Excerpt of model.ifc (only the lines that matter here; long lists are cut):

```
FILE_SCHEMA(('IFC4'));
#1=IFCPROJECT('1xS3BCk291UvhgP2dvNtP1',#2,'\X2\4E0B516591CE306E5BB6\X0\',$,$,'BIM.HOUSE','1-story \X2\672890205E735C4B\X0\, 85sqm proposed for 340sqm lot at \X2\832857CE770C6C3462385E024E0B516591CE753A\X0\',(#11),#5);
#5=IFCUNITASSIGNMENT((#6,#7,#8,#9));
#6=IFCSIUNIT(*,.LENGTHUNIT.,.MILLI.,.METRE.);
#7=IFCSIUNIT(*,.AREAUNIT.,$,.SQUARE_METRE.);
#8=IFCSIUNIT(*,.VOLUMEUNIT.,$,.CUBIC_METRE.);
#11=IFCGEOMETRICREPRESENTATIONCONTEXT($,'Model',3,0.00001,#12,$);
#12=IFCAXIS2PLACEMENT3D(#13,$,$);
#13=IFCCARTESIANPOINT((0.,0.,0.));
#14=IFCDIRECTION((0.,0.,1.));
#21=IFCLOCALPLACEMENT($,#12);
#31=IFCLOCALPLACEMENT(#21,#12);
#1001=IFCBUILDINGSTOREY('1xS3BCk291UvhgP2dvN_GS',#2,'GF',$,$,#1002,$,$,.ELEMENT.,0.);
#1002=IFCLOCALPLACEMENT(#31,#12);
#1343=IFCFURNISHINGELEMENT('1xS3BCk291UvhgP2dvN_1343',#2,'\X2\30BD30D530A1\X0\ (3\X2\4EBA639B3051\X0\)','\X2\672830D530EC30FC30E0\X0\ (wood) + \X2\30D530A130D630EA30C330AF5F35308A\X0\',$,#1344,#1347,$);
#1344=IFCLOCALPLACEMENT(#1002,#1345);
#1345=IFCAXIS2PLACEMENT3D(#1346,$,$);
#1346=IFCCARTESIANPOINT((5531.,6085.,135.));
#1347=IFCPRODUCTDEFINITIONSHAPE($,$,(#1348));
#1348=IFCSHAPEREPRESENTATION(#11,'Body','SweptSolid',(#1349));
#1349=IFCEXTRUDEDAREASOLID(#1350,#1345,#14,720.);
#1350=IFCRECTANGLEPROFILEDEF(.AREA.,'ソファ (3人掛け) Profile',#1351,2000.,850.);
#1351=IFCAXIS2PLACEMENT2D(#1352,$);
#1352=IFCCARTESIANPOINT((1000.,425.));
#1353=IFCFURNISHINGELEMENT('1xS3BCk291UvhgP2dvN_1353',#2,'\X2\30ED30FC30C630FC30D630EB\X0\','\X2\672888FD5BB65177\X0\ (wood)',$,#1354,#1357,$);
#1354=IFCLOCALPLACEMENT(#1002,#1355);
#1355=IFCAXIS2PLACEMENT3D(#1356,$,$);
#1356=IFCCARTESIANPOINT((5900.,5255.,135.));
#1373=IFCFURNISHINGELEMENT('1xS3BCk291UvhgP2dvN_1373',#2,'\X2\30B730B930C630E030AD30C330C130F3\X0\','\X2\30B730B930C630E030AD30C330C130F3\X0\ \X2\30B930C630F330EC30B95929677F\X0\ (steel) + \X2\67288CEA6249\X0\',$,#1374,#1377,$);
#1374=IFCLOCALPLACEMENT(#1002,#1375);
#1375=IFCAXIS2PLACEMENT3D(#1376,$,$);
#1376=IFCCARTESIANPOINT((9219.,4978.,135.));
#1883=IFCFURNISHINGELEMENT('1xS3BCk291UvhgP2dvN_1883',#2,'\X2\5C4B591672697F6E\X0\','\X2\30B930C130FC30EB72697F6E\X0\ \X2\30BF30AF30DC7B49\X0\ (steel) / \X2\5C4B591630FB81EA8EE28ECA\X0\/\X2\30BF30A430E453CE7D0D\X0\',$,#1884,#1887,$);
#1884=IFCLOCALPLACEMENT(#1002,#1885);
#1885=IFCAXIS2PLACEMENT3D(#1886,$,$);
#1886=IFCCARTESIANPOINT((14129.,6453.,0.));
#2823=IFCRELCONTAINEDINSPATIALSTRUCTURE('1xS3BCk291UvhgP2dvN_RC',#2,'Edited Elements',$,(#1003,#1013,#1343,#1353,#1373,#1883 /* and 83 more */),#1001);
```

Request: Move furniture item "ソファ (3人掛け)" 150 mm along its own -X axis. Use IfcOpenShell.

```python
import ifcopenshell
import ifcopenshell.api.geometry
import ifcopenshell.util.placement
import ifcopenshell.util.unit

model = ifcopenshell.open("model.ifc")
unit_scale = ifcopenshell.util.unit.calculate_unit_scale(model)

item = model.by_guid("1xS3BCk291UvhgP2dvN_1343")
matrix = ifcopenshell.util.placement.get_local_placement(item.ObjectPlacement)
matrix[:3, 3] -= matrix[:3, 0] * 0.15 / unit_scale
ifcopenshell.api.geometry.edit_object_placement(model, product=item, matrix=matrix, is_si=False)

print(ifcopenshell.util.placement.get_local_placement(item.ObjectPlacement).round(3) + 0.0)

model.write("model_rev.ifc")
```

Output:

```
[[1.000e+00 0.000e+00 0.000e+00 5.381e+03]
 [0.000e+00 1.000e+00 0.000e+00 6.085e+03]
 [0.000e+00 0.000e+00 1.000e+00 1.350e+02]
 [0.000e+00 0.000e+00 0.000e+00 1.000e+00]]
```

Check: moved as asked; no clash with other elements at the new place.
